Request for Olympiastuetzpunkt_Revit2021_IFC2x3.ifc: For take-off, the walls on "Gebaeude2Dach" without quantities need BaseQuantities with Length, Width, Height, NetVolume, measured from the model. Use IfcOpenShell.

First a look at what the model holds.

```python
import ifcopenshell
import ifcopenshell.util.element
import ifcopenshell.util.unit

model = ifcopenshell.open("Olympiastuetzpunkt_Revit2021_IFC2x3.ifc")
print(model.schema)
for unit_type in ("LENGTHUNIT", "AREAUNIT", "VOLUMEUNIT"):
    print(unit_type, ifcopenshell.util.unit.calculate_unit_scale(model, unit_type))
storey = next(s for s in model.by_type("IfcBuildingStorey") if s.Name == "Gebaeude2Dach")
walls = [e for e in ifcopenshell.util.element.get_decomposition(storey) if e.is_a("IfcWall")]
for e in sorted(walls, key=lambda e: e.id()):
    print(e.id(), e.is_a(), e.Name, list(ifcopenshell.util.element.get_psets(e, qtos_only=True)), sep=" | ")
```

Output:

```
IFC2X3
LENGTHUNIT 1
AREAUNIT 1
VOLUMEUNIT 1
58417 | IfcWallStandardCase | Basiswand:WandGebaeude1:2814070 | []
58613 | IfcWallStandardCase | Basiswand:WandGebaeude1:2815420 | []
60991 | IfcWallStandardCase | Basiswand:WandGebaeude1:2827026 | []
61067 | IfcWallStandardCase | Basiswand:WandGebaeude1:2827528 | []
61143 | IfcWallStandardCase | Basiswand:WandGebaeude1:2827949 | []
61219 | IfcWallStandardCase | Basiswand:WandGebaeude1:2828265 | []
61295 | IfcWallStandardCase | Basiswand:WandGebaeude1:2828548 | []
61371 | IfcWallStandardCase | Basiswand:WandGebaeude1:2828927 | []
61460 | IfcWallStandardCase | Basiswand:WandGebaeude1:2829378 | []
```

```python
import ifcopenshell
import ifcopenshell.api.pset
import ifcopenshell.geom
import ifcopenshell.util.element
import ifcopenshell.util.shape
import ifcopenshell.util.unit

model = ifcopenshell.open("Olympiastuetzpunkt_Revit2021_IFC2x3.ifc")
unit_scale = ifcopenshell.util.unit.calculate_unit_scale(model)
volume_scale = ifcopenshell.util.unit.calculate_unit_scale(model, "VOLUMEUNIT")
settings = ifcopenshell.geom.settings()

storey = next(s for s in model.by_type("IfcBuildingStorey") if s.Name == "Gebaeude2Dach")
walls = [e for e in ifcopenshell.util.element.get_decomposition(storey) if e.is_a("IfcWall")]

for e in sorted(walls, key=lambda e: e.id()):
    if ifcopenshell.util.element.get_psets(e, qtos_only=True, should_inherit=False):
        continue
    # Geometry comes back in metres, in the element's own axes.
    shape = ifcopenshell.geom.create_shape(settings, e)
    values = {
        "Length": ifcopenshell.util.shape.get_x(shape.geometry) / unit_scale,
        "Width": ifcopenshell.util.shape.get_y(shape.geometry) / unit_scale,
        "Height": ifcopenshell.util.shape.get_z(shape.geometry) / unit_scale,
        "NetVolume": ifcopenshell.util.shape.get_volume(shape.geometry) / volume_scale,
    }
    qto = ifcopenshell.api.pset.add_qto(model, product=e, name="BaseQuantities")
    ifcopenshell.api.pset.edit_qto(model, qto=qto, properties=values)
    print(e.id(), {k: round(v, 3) for k, v in values.items()})

model.write("Olympiastuetzpunkt_Revit2021_IFC2x3_rev.ifc")
```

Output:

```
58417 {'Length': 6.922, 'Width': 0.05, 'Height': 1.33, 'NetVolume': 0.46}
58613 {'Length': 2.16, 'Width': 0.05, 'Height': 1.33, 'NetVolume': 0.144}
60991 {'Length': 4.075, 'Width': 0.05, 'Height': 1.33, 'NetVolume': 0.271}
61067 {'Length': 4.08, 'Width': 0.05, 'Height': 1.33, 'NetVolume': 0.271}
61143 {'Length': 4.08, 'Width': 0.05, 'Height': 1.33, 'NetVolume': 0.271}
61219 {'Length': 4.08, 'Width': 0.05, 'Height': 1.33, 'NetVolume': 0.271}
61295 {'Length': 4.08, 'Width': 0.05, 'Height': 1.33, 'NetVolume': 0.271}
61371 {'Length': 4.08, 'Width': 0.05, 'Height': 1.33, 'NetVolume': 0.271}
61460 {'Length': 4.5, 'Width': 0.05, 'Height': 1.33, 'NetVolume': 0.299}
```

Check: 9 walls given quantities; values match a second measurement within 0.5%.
